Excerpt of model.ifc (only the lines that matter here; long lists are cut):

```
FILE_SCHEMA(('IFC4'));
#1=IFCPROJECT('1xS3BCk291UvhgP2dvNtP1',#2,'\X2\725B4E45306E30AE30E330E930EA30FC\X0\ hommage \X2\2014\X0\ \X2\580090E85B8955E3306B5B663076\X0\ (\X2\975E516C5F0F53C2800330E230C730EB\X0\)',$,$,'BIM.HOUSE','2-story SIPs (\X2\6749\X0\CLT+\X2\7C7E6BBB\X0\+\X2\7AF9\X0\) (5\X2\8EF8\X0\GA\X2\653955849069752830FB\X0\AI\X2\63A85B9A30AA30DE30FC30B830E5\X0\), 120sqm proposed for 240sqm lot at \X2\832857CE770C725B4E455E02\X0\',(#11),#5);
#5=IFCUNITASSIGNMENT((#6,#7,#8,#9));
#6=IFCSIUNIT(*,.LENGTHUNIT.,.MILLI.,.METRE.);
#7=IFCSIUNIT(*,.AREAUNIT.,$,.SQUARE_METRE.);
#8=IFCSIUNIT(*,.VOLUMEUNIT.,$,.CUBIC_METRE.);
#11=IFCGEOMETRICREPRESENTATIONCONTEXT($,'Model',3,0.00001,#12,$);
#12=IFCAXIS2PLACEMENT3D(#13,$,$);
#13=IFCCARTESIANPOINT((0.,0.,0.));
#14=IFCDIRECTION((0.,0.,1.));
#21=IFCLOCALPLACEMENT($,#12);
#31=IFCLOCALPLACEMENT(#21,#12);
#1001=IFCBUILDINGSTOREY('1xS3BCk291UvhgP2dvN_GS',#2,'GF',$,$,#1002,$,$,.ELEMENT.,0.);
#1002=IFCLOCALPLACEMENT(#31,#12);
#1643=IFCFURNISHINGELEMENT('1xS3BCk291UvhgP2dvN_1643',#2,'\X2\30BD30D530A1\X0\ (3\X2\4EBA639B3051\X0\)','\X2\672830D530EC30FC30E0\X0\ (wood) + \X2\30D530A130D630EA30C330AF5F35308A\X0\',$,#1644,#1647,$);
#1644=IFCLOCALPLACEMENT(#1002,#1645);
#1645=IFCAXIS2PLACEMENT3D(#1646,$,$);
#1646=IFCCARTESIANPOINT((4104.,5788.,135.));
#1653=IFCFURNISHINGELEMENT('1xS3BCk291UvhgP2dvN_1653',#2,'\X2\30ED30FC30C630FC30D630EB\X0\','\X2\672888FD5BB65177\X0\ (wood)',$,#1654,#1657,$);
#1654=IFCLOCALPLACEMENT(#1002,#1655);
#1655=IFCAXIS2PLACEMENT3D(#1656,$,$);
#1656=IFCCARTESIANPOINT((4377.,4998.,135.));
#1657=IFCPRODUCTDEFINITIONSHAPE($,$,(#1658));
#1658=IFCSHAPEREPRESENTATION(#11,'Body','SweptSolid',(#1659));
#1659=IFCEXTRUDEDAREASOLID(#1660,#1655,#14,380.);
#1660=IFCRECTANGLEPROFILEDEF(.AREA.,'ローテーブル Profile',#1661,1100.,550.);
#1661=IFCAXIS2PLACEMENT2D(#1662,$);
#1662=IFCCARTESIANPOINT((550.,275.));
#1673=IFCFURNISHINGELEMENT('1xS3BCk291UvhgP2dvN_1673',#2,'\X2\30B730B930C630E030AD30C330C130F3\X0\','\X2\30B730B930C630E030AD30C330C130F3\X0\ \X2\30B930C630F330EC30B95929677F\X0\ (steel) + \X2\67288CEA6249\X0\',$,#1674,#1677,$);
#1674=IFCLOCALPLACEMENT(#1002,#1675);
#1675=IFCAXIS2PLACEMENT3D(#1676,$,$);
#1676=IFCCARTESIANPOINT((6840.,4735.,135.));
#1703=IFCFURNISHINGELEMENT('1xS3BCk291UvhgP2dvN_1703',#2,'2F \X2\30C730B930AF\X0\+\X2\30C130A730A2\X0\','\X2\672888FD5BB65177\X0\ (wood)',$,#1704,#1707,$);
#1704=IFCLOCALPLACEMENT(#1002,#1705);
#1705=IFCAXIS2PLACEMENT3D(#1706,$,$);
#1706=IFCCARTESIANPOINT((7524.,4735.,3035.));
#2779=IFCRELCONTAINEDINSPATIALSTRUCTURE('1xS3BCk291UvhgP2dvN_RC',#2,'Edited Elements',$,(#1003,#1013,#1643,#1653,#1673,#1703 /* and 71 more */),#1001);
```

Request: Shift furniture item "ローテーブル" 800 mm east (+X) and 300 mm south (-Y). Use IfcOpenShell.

```python
import ifcopenshell
import ifcopenshell.api.geometry
import ifcopenshell.util.placement

model = ifcopenshell.open("model.ifc")

item = model.by_guid("1xS3BCk291UvhgP2dvN_1653")
matrix = ifcopenshell.util.placement.get_local_placement(item.ObjectPlacement)
matrix[0, 3] += 800.0
matrix[1, 3] -= 300.0
ifcopenshell.api.geometry.edit_object_placement(model, product=item, matrix=matrix, is_si=False)

print(ifcopenshell.util.placement.get_local_placement(item.ObjectPlacement).round(3) + 0.0)

model.write("model_rev.ifc")
```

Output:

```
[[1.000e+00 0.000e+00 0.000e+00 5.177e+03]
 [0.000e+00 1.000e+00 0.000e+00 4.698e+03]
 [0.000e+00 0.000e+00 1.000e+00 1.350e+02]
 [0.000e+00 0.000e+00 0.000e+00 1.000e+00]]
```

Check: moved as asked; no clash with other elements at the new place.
